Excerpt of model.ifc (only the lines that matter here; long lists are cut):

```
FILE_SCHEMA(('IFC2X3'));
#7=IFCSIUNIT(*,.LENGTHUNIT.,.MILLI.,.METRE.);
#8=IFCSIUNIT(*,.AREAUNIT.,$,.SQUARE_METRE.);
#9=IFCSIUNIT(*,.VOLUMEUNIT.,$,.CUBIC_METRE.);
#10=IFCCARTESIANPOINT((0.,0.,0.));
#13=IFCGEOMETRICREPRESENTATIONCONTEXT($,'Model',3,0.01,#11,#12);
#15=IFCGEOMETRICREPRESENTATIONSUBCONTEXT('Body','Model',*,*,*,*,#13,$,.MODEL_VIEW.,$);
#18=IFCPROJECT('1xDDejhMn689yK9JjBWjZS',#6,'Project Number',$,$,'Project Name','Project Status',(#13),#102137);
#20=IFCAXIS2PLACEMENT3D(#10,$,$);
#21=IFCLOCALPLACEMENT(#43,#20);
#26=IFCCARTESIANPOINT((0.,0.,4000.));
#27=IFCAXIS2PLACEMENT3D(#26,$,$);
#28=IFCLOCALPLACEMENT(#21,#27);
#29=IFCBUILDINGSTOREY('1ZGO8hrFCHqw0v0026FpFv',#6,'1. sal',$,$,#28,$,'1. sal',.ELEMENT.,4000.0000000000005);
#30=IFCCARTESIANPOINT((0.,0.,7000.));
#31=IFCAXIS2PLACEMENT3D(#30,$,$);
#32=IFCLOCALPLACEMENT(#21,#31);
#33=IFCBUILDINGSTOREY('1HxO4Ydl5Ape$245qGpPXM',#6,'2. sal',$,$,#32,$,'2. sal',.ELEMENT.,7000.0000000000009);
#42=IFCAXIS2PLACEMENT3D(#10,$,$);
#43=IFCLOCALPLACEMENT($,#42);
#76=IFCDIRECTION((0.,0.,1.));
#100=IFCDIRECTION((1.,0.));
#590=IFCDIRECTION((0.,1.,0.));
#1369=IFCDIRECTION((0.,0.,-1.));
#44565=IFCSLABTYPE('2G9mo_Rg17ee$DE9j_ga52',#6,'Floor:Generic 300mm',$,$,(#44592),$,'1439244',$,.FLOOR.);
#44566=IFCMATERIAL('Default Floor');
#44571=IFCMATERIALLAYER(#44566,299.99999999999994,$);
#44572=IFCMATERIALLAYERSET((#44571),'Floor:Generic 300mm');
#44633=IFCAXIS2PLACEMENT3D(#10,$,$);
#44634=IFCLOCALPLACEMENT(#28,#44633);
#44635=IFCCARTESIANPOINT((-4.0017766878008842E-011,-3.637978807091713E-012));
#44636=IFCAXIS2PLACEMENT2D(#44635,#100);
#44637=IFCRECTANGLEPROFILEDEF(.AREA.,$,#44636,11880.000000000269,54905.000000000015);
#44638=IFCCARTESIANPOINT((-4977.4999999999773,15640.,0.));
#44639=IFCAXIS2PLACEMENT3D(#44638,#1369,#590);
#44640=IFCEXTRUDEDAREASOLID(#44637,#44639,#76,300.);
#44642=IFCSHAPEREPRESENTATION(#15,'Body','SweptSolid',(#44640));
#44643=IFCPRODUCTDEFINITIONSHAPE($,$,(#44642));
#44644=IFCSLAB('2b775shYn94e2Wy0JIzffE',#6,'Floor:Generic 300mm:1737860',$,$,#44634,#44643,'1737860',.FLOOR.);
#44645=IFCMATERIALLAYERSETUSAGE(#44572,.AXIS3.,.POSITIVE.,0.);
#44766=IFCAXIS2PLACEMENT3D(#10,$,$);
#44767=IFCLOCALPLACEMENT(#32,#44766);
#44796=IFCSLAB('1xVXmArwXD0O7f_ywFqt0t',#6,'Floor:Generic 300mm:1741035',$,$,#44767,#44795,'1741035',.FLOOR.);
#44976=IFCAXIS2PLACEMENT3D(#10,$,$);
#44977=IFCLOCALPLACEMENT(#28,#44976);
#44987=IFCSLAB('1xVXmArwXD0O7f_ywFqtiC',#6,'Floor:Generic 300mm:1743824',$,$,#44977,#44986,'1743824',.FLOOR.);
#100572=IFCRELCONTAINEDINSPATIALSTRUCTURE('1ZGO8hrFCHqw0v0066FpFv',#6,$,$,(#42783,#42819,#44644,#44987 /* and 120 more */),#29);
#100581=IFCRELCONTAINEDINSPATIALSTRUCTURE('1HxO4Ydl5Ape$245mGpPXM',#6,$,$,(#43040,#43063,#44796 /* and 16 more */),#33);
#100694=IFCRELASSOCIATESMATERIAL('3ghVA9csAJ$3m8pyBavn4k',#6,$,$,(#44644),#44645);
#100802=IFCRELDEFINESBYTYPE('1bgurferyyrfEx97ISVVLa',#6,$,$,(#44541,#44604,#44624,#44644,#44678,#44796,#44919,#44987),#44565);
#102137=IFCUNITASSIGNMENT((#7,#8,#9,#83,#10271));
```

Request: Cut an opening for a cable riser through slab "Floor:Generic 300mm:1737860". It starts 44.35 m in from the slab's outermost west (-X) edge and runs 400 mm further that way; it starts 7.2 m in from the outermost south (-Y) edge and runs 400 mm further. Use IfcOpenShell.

```python
import numpy as np
import ifcopenshell
import ifcopenshell.api.feature
import ifcopenshell.api.geometry
import ifcopenshell.api.root
import ifcopenshell.geom
import ifcopenshell.util.placement
import ifcopenshell.util.representation
import ifcopenshell.util.shape
import ifcopenshell.util.unit

model = ifcopenshell.open("model.ifc")
unit_scale = ifcopenshell.util.unit.calculate_unit_scale(model)
settings = ifcopenshell.geom.settings()


def volume(element):
    """Net volume in cubic metres, openings subtracted."""
    shape = ifcopenshell.geom.create_shape(settings, element)
    return ifcopenshell.util.shape.get_volume(shape.geometry)


slab = model.by_guid("2b775shYn94e2Wy0JIzffE")
before = volume(slab)

# Extent in the slab's own axes, in metres. The edges named are its -X and -Y sides.
slab_shape = ifcopenshell.geom.create_shape(settings, slab)
vertices = ifcopenshell.util.shape.get_vertices(slab_shape.geometry)
x_min, y_min, bottom = vertices.min(axis=0)
top = vertices[:, 2].max()

opening = ifcopenshell.api.root.create_entity(model, ifc_class="IfcOpeningElement", name="Cable riser opening")
context = ifcopenshell.util.representation.get_context(model, "Model", "Body", "MODEL_VIEW")
width, depth = 0.4, 0.4
outline = [(0.0, 0.0), (width, 0.0), (width, depth), (0.0, depth), (0.0, 0.0)]
# Overshoot both faces by 50 mm so the cut is clean.
shape = ifcopenshell.api.geometry.add_slab_representation(
    model, context=context, depth=top - bottom + 0.1, polyline=outline
)
ifcopenshell.api.geometry.assign_representation(model, product=opening, representation=shape)

matrix = ifcopenshell.util.placement.get_local_placement(slab.ObjectPlacement)
matrix[:, 3] = matrix @ np.append(np.array([x_min + 44.35, y_min + 7.2, bottom - 0.05]) / unit_scale, 1.0)
ifcopenshell.api.geometry.edit_object_placement(model, product=opening, matrix=matrix, is_si=False)
ifcopenshell.api.feature.add_feature(model, feature=opening, element=slab)

after = volume(slab)

print(f"slab volume {before:.3f} -> {after:.3f} m3")

model.write("model_updated.ifc")
```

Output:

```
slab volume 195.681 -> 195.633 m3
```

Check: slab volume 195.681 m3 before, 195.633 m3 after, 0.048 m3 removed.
